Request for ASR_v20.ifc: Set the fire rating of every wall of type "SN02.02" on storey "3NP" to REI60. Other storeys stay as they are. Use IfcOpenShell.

First a look at what the model holds.

```python
import ifcopenshell
import ifcopenshell.util.element

model = ifcopenshell.open("ASR_v20.ifc")
print(model.schema)
storey = next(s for s in model.by_type("IfcBuildingStorey") if s.Name == "3NP")
walls = [e for e in ifcopenshell.util.element.get_decomposition(storey) if e.is_a("IfcWall")]
seen = {}
for e in walls:
    element_type = ifcopenshell.util.element.get_type(e)
    key = (element_type.Name if element_type != e and element_type else None, ifcopenshell.util.element.get_pset(e, "Pset_WallCommon", "FireRating"))
    seen[key] = seen.get(key, 0) + 1
for (name, value), count in sorted(seen.items(), key=str):
    print(count, "x", name, "|", value)
```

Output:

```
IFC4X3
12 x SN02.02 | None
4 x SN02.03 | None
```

```python
import ifcopenshell
import ifcopenshell.api.pset
import ifcopenshell.util.element

model = ifcopenshell.open("ASR_v20.ifc")

storey = next(s for s in model.by_type("IfcBuildingStorey") if s.Name == "3NP")
walls = [e for e in ifcopenshell.util.element.get_decomposition(storey) if e.is_a("IfcWall")]

count = 0
for e in walls:
    element_type = ifcopenshell.util.element.get_type(e)
    if element_type in (None, e) or element_type.Name != "SN02.02":
        continue
    # add_pset returns the element's existing set when there is one.
    pset = ifcopenshell.api.pset.add_pset(model, product=e, name="Pset_WallCommon")
    ifcopenshell.api.pset.edit_pset(model, pset=pset, properties={"FireRating": "REI60"})
    count += 1

print(count, "walls updated")

model.write("ASR_v20_edited.ifc")
```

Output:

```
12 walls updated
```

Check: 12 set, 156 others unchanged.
